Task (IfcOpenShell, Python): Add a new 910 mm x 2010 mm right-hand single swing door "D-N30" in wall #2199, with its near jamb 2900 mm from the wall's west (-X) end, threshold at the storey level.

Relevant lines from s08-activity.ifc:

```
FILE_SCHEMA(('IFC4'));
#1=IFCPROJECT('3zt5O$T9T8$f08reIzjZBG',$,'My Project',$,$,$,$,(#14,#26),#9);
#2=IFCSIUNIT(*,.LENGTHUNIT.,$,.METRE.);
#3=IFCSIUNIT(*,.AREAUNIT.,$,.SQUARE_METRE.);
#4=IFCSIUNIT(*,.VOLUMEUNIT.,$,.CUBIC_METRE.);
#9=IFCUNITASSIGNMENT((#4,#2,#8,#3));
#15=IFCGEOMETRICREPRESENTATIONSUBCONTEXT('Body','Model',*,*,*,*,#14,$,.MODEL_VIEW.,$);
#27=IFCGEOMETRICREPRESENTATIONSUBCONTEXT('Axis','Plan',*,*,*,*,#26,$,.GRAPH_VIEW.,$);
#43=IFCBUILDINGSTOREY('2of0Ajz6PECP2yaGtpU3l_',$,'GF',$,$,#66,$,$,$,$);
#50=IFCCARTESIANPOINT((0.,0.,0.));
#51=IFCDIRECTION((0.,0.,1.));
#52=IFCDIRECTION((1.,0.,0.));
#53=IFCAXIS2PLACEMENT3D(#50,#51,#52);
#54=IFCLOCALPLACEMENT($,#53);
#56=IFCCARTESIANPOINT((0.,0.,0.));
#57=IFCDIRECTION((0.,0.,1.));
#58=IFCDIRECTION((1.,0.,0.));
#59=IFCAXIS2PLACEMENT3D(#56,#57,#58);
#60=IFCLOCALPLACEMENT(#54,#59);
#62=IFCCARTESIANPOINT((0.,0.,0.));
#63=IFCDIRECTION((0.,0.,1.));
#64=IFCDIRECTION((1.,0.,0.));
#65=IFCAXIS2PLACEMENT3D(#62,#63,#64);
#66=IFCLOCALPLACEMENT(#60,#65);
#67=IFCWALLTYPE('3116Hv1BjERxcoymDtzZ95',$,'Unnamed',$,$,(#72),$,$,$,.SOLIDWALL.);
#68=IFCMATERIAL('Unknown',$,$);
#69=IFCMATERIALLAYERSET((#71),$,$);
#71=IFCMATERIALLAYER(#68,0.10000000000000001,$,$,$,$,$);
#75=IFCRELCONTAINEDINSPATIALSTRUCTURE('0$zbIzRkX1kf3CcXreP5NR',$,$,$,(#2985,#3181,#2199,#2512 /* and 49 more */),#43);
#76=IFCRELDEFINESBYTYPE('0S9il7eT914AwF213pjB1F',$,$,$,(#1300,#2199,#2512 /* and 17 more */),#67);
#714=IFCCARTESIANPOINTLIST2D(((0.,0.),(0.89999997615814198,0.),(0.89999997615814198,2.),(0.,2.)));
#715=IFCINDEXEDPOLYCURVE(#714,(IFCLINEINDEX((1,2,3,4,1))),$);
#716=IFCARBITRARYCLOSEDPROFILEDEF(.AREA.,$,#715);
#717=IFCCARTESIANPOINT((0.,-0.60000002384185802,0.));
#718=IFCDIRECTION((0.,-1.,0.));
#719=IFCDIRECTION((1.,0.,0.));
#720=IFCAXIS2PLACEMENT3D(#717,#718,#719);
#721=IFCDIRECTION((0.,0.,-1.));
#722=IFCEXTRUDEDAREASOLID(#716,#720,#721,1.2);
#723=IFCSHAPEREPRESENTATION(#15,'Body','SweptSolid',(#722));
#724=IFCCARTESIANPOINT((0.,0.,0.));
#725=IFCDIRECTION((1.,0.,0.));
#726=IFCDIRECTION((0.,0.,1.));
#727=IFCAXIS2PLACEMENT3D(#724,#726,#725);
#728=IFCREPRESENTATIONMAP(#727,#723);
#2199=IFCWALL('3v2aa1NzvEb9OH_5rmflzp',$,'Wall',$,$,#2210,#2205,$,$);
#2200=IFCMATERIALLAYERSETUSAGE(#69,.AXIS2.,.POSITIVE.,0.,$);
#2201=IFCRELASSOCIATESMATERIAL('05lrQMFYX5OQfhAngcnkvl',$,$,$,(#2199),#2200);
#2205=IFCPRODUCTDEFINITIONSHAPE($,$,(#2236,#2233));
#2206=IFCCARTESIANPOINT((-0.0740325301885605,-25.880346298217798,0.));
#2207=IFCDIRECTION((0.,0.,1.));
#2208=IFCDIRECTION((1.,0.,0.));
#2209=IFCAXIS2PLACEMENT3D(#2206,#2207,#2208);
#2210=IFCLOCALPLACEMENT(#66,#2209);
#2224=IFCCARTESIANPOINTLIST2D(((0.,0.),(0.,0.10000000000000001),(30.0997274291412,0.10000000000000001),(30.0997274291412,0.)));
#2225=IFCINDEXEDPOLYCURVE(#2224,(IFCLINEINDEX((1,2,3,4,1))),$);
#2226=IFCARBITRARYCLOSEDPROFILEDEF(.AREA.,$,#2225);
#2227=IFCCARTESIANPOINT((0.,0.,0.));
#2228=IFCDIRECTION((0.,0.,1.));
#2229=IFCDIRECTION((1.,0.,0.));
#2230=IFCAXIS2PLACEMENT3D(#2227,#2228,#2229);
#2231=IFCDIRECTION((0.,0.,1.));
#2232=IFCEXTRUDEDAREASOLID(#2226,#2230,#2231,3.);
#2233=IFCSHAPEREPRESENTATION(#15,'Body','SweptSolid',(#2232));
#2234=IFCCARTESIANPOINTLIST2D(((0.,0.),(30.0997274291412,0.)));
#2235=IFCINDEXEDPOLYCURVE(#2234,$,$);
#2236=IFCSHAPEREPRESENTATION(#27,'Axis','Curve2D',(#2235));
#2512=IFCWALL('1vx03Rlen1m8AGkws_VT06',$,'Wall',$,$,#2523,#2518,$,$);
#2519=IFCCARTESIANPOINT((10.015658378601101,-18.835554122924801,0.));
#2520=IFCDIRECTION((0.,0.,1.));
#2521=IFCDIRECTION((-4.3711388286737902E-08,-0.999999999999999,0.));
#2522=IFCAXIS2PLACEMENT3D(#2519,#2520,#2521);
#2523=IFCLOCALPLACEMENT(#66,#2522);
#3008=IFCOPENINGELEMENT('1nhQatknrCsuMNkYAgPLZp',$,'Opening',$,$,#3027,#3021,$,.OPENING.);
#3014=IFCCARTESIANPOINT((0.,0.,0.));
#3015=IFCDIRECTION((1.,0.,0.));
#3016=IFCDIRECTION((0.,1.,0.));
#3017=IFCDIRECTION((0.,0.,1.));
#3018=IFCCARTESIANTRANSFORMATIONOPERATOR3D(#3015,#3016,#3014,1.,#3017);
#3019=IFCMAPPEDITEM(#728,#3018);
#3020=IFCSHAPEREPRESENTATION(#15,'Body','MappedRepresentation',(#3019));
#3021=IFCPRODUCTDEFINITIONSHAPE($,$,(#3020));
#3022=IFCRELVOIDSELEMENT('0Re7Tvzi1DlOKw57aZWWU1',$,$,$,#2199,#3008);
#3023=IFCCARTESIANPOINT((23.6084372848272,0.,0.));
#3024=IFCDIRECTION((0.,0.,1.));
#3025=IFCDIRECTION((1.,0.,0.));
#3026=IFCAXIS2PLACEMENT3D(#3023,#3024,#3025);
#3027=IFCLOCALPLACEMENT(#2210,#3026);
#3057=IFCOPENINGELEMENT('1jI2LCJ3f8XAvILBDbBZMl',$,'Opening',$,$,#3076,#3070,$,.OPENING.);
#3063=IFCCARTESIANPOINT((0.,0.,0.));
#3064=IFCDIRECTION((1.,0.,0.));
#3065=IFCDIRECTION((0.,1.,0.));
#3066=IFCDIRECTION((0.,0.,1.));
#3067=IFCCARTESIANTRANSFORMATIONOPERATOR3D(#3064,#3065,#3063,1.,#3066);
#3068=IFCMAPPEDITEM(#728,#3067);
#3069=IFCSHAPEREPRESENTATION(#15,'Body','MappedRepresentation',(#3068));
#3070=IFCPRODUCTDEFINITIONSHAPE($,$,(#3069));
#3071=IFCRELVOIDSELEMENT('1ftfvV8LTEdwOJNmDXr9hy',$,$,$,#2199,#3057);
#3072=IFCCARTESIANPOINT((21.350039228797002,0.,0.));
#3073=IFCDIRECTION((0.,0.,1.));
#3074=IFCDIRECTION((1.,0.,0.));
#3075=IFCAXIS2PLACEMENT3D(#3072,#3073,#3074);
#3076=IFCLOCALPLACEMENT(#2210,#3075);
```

```python
import numpy as np
import ifcopenshell
import ifcopenshell.api.feature
import ifcopenshell.api.geometry
import ifcopenshell.api.root
import ifcopenshell.api.spatial
import ifcopenshell.geom
import ifcopenshell.util.element
import ifcopenshell.util.placement
import ifcopenshell.util.representation
import ifcopenshell.util.shape
import ifcopenshell.util.unit

model = ifcopenshell.open("s08-activity.ifc")
unit_scale = ifcopenshell.util.unit.calculate_unit_scale(model)
settings = ifcopenshell.geom.settings()


def volume(element):
    """Net volume in cubic metres, openings subtracted."""
    shape = ifcopenshell.geom.create_shape(settings, element)
    return ifcopenshell.util.shape.get_volume(shape.geometry)


wall = model.by_guid("3v2aa1NzvEb9OH_5rmflzp")
storey = ifcopenshell.util.element.get_container(wall, ifc_class="IfcBuildingStorey")
context = ifcopenshell.util.representation.get_context(model, "Model", "Body", "MODEL_VIEW")
before = volume(wall)

width, height, from_end, sill = 0.91, 2.01, 2.9, 0.0  # metres

# The wall runs along its own X axis, and the end named is its -X end.
wall_shape = ifcopenshell.geom.create_shape(settings, wall)
x, y, z = ifcopenshell.util.shape.get_vertices(wall_shape.geometry).T
start = x.min() + from_end
face, thickness = float(y.min()), float(y.max() - y.min())
wall_matrix = ifcopenshell.util.placement.get_local_placement(wall.ObjectPlacement)
level = ifcopenshell.util.placement.get_local_placement(storey.ObjectPlacement)[2, 3]


def in_wall(x, y):
    """Placement at x, y metres in the wall's axes, at sill height."""
    matrix = wall_matrix.copy()
    matrix[:, 3] = wall_matrix @ np.array([x / unit_scale, y / unit_scale, 0.0, 1.0])
    matrix[2, 3] = level + sill / unit_scale
    return matrix


# Opening: a box that overshoots both wall faces by 50 mm.
opening = ifcopenshell.api.root.create_entity(model, ifc_class="IfcOpeningElement", predefined_type="OPENING")
box = ifcopenshell.api.geometry.add_wall_representation(
    model, context=context, length=width, height=height, thickness=thickness + 0.1
)
ifcopenshell.api.geometry.assign_representation(model, product=opening, representation=box)
ifcopenshell.api.geometry.edit_object_placement(model, product=opening, matrix=in_wall(start, face - 0.05), is_si=False)
ifcopenshell.api.feature.add_feature(model, feature=opening, element=wall)

door = ifcopenshell.api.root.create_entity(model, ifc_class="IfcDoor", name="D-N30", predefined_type="DOOR")
door.OverallWidth, door.OverallHeight = width / unit_scale, height / unit_scale
door.OperationType = "SINGLE_SWING_RIGHT"
body = ifcopenshell.api.geometry.add_door_representation(
    model,
    context=context,
    overall_width=door.OverallWidth,
    overall_height=door.OverallHeight,
    operation_type="SINGLE_SWING_RIGHT",
    lining_properties={"LiningDepth": thickness / unit_scale, "ThresholdDepth": thickness / unit_scale},
)
ifcopenshell.api.geometry.assign_representation(model, product=door, representation=body)
ifcopenshell.api.spatial.assign_container(model, products=[door], relating_structure=storey)
ifcopenshell.api.feature.add_filling(model, opening=opening, element=door)

# The lining spans the wall, so the door starts at the wall face.
ifcopenshell.api.geometry.edit_object_placement(model, product=door, matrix=in_wall(start, face), is_si=False)

after = volume(wall)

print(f"wall volume {before:.3f} -> {after:.3f} m3")

model.write("s08-activity_rev.ifc")
```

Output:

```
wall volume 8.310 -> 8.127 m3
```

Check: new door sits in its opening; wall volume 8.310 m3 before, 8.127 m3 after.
